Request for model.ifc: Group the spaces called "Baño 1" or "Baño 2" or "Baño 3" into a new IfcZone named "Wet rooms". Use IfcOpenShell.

First a look at what the model holds.

```python
import ifcopenshell

model = ifcopenshell.open("model.ifc")
print(model.schema)
seen = {}
for space in model.by_type("IfcSpace"):
    seen[space.LongName] = seen.get(space.LongName, 0) + 1
for name, count in sorted(seen.items(), key=str):
    print(count, "x", name)
print("zones:", [z.Name for z in model.by_type("IfcZone")][:20])
```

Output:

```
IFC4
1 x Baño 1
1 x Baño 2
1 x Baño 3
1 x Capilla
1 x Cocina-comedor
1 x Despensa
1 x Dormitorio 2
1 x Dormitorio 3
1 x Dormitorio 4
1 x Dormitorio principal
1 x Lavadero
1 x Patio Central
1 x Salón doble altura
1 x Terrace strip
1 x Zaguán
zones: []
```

```python
import ifcopenshell
import ifcopenshell.api.group
import ifcopenshell.api.root

model = ifcopenshell.open("model.ifc")

names = {"Baño 1", "Baño 2", "Baño 3"}
spaces = [s for s in model.by_type("IfcSpace") if s.LongName in names]

zone = ifcopenshell.api.root.create_entity(model, ifc_class="IfcZone", name="Wet rooms")
ifcopenshell.api.group.assign_group(model, products=spaces, group=zone)
print(len(spaces), "spaces in", zone.Name)

model.write("model_updated.ifc")
```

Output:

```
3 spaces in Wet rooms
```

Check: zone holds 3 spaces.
